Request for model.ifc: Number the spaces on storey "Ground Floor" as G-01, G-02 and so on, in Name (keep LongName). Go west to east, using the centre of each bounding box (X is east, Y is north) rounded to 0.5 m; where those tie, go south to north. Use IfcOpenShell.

First a look at what the model holds.

```python
import ifcopenshell
import ifcopenshell.util.element
import ifcopenshell.util.placement

model = ifcopenshell.open("model.ifc")
print(model.schema)
storey = next(s for s in model.by_type("IfcBuildingStorey") if s.Name == "Ground Floor")
spaces = [e for e in ifcopenshell.util.element.get_decomposition(storey) if e.is_a("IfcSpace")]
for e in sorted(spaces, key=lambda e: e.id()):
    origin = ifcopenshell.util.placement.get_local_placement(e.ObjectPlacement)[:3, 3]
    print(e.id(), e.Name, e.LongName, origin.round(2) + 0.0, sep=" | ")
```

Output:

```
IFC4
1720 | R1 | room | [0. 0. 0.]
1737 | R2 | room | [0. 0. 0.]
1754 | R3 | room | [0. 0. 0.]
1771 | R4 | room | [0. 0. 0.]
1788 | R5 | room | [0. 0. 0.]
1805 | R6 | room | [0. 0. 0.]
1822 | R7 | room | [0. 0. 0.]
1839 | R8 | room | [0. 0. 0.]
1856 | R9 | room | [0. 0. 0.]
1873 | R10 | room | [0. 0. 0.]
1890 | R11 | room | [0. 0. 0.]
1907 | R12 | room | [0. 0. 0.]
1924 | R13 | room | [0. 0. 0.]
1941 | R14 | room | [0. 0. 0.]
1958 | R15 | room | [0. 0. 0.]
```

```python
import ifcopenshell
import ifcopenshell.geom
import ifcopenshell.util.element
import ifcopenshell.util.shape

model = ifcopenshell.open("model.ifc")
settings = ifcopenshell.geom.settings()
settings.set("use-world-coords", True)


def centre(element):
    shape = ifcopenshell.geom.create_shape(settings, element)
    return ifcopenshell.util.shape.get_bbox_centroid(shape.geometry)


storey = next(s for s in model.by_type("IfcBuildingStorey") if s.Name == "Ground Floor")
spaces = [e for e in ifcopenshell.util.element.get_decomposition(storey) if e.is_a("IfcSpace")]

# Insertion points can sit at a corner or the storey origin, so sort by the geometry (in metres).
centres = {e: centre(e) for e in spaces}
spaces.sort(key=lambda e: (round(centres[e][0] / 0.5), centres[e][1]))

for i, e in enumerate(spaces, start=1):
    number = f"G-{i:02d}"
    e.Name = number
    print(e.id(), number)

model.write("model_edited.ifc")
```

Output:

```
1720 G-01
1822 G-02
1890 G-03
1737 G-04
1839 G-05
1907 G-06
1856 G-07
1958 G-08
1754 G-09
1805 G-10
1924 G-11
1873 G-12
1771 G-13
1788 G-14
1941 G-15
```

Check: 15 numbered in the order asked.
